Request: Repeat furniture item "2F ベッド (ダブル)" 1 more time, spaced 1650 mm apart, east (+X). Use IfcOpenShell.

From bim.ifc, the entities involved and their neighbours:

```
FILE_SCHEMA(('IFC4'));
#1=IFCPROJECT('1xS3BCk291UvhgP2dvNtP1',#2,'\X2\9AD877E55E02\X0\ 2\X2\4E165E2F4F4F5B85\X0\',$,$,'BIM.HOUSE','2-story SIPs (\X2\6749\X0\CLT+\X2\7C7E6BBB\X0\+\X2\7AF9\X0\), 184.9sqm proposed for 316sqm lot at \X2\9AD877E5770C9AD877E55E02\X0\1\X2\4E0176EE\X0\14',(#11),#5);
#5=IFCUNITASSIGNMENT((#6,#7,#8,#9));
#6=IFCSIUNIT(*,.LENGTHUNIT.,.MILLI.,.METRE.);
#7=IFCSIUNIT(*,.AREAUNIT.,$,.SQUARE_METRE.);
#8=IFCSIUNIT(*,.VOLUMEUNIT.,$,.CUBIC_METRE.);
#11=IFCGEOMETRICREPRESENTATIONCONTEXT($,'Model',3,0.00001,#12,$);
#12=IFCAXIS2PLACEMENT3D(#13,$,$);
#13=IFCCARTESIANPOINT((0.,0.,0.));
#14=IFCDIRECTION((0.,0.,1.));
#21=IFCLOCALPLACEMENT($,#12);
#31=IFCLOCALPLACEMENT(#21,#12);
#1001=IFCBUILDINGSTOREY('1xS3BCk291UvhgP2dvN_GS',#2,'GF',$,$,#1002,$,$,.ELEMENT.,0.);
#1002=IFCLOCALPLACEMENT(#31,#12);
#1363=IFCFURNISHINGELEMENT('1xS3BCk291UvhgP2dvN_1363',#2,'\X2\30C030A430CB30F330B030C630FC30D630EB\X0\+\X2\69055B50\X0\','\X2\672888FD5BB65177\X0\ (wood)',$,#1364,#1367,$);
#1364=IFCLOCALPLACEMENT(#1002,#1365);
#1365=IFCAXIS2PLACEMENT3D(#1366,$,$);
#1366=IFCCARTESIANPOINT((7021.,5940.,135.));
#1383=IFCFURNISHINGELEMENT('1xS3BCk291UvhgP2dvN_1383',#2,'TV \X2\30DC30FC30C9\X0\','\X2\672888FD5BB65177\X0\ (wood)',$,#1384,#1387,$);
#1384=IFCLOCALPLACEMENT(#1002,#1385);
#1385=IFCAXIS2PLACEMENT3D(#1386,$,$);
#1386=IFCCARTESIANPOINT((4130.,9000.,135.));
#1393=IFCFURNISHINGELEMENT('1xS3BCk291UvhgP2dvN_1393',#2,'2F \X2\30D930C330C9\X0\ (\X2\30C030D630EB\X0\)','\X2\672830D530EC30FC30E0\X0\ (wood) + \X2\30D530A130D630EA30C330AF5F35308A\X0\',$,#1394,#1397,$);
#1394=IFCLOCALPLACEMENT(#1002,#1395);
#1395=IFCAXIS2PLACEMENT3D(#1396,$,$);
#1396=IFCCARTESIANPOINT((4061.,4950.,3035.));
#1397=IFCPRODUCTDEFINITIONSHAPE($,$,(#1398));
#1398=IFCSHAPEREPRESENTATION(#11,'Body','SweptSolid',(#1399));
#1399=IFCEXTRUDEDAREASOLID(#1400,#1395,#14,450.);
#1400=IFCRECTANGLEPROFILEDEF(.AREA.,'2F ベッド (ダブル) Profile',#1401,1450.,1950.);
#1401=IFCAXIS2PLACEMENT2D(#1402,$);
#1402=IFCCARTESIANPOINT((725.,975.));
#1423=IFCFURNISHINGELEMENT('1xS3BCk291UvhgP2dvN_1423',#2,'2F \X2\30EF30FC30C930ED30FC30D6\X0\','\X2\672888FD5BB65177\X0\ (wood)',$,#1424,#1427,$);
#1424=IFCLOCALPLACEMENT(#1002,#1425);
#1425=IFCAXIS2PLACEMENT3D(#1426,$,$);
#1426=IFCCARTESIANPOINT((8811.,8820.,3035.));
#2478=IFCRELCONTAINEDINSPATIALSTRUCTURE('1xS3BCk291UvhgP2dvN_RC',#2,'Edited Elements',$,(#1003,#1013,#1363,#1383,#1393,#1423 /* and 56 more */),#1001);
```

```python
import numpy as np
import ifcopenshell
import ifcopenshell.api.geometry
import ifcopenshell.api.root
import ifcopenshell.util.element
import ifcopenshell.util.placement

model = ifcopenshell.open("bim.ifc")


def reuse_history(source, copy):
    """copy_class also copies each property set's owner history, people and application; keep the originals."""
    for rel in copy.IsDefinedBy:
        if rel.is_a("IfcRelDefinesByProperties") and (history := rel.RelatingPropertyDefinition.OwnerHistory):
            rel.RelatingPropertyDefinition.OwnerHistory = source.OwnerHistory
            ifcopenshell.util.element.remove_deep2(model, history)


source = model.by_guid("1xS3BCk291UvhgP2dvN_1393")
base = ifcopenshell.util.placement.get_local_placement(source.ObjectPlacement)
step = np.array([1.0, 0.0, 0.0]) * 1650.0

for i in range(1, 2):
    copy = ifcopenshell.api.root.copy_class(model, product=source)
    copy.Representation = ifcopenshell.util.element.copy_deep(
        model, source.Representation, exclude=["IfcGeometricRepresentationContext", "IfcRepresentationMap"]
    )
    reuse_history(source, copy)
    matrix = base.copy()
    matrix[:3, 3] += i * step
    print("added at", matrix[:3, 3].round(3) + 0.0)
    ifcopenshell.api.geometry.edit_object_placement(model, product=copy, matrix=matrix, is_si=False)

model.write("bim_updated.ifc")
```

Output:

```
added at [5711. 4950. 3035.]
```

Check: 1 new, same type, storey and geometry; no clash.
